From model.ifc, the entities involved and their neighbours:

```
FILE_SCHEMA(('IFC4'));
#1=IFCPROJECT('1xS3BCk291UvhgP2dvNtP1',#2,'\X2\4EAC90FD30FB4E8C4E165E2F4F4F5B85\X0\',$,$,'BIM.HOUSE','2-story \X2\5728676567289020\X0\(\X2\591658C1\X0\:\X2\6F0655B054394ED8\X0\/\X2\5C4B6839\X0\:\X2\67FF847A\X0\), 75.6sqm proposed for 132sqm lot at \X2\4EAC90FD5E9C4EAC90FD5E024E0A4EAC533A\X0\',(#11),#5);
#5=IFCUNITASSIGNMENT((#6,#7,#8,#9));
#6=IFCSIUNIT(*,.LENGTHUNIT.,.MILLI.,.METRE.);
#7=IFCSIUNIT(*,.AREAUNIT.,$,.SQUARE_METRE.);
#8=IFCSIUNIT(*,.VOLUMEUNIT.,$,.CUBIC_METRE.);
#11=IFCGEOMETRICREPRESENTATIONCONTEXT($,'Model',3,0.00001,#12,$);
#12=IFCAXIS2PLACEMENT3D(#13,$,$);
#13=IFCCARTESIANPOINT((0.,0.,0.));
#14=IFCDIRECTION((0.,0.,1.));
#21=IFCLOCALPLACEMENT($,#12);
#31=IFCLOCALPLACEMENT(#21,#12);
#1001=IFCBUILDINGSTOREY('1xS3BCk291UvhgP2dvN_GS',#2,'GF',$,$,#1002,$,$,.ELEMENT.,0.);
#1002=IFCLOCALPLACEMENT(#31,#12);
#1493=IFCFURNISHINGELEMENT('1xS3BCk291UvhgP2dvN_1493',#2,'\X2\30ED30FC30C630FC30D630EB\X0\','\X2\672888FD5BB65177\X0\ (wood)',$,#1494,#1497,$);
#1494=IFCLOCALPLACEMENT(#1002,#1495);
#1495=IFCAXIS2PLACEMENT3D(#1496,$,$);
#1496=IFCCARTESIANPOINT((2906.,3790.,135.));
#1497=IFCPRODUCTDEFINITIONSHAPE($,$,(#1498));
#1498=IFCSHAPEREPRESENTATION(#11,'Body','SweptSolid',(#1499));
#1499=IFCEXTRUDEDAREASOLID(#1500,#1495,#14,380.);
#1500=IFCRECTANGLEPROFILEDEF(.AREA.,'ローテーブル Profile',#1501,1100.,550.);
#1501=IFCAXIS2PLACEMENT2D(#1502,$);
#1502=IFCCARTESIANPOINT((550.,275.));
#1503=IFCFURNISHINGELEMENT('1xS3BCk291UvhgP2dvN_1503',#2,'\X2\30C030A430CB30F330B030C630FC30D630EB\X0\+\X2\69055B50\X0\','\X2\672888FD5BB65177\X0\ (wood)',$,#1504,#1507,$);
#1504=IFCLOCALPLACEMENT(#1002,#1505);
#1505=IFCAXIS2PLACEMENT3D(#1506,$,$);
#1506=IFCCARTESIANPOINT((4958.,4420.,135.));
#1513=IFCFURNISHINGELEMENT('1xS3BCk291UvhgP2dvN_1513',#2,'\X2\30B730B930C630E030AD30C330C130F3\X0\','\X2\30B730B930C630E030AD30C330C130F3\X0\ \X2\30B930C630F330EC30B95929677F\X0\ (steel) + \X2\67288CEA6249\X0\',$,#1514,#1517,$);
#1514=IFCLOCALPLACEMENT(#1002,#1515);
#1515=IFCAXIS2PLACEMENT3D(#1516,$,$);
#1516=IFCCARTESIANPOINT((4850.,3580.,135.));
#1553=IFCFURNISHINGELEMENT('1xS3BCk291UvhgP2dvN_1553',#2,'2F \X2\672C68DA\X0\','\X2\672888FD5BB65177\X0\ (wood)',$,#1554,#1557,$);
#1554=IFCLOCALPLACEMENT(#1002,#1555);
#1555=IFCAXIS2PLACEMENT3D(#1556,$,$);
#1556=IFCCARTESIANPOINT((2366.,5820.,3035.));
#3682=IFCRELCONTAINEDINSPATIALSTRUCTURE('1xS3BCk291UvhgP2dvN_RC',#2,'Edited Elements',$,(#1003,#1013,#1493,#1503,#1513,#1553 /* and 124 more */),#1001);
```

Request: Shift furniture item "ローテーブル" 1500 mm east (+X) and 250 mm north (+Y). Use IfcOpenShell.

```python
import ifcopenshell
import ifcopenshell.api.geometry
import ifcopenshell.util.placement
import ifcopenshell.util.unit

model = ifcopenshell.open("model.ifc")
unit_scale = ifcopenshell.util.unit.calculate_unit_scale(model)

item = model.by_guid("1xS3BCk291UvhgP2dvN_1493")
matrix = ifcopenshell.util.placement.get_local_placement(item.ObjectPlacement)
matrix[0, 3] += 1.5 / unit_scale
matrix[1, 3] += 0.25 / unit_scale
ifcopenshell.api.geometry.edit_object_placement(model, product=item, matrix=matrix, is_si=False)

print(ifcopenshell.util.placement.get_local_placement(item.ObjectPlacement).round(3) + 0.0)

model.write("model_updated.ifc")
```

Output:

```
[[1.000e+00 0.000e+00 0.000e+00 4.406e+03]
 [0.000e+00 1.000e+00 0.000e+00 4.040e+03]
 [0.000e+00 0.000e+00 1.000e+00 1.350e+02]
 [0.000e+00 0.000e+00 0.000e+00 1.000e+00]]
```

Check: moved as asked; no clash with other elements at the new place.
